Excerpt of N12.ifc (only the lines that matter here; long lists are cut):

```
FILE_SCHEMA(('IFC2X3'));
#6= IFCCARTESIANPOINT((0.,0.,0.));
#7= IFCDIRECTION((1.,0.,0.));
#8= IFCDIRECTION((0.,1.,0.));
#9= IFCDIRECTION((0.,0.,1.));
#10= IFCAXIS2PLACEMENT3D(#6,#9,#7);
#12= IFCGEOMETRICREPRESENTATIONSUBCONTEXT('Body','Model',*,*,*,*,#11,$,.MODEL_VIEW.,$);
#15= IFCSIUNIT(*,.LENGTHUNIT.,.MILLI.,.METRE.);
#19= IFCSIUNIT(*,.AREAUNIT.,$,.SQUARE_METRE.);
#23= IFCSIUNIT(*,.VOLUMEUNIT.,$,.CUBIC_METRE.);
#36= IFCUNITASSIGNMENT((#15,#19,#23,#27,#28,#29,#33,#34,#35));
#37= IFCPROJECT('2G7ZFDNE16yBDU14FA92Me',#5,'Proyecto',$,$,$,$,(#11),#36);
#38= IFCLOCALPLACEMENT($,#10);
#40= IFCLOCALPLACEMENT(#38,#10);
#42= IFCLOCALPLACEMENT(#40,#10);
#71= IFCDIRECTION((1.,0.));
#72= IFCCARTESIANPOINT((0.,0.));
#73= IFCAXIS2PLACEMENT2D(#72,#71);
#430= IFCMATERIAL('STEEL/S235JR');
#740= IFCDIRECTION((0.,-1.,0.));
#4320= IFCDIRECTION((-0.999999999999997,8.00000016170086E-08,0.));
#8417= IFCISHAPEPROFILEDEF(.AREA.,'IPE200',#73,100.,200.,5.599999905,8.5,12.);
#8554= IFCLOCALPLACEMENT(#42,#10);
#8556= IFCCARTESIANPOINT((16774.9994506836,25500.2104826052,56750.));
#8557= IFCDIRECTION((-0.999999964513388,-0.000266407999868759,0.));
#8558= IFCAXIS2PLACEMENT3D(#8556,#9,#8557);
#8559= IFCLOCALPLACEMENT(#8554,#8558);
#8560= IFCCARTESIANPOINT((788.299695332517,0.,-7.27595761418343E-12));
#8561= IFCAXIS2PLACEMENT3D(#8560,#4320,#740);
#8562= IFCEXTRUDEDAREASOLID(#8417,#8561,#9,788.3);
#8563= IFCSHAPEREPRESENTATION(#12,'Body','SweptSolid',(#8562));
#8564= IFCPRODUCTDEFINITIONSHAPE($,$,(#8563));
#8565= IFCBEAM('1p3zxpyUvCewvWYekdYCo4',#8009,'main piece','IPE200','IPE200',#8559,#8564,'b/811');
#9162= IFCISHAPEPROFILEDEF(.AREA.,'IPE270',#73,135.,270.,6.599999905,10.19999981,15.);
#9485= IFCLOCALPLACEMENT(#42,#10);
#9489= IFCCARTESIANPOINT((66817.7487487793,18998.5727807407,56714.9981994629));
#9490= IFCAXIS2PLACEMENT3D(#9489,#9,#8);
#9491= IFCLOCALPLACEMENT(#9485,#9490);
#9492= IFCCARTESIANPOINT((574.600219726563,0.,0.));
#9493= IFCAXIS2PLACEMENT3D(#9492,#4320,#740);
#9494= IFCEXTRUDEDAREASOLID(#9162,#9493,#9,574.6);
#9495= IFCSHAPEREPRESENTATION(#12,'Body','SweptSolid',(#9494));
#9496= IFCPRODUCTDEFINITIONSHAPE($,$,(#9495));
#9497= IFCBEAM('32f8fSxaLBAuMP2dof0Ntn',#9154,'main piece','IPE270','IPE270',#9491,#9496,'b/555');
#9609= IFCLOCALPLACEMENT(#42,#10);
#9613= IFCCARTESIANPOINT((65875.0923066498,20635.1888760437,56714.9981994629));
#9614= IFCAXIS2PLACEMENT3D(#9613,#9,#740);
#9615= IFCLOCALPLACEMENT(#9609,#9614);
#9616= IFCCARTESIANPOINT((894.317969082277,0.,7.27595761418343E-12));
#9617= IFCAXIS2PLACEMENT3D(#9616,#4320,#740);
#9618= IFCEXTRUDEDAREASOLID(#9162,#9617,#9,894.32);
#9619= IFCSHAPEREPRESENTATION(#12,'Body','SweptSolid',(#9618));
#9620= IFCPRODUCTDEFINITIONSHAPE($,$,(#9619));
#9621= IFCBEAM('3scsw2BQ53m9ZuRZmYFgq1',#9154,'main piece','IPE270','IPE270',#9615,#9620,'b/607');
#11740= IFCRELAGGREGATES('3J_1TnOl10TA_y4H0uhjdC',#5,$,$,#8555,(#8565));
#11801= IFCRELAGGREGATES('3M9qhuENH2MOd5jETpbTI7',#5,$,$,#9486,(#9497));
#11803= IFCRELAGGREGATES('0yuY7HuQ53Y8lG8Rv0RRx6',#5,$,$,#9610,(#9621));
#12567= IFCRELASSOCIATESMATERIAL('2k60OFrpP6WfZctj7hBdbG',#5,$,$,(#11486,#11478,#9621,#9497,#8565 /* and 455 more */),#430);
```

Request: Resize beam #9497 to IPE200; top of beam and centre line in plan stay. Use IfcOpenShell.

```python
import ifcopenshell
import ifcopenshell.util.element
import ifcopenshell.util.representation

model = ifcopenshell.open("N12.ifc")

member = model.by_guid("32f8fSxaLBAuMP2dof0Ntn")
source = next(p for p in model.by_type("IfcIShapeProfileDef") if p.ProfileName == "IPE200")

body = ifcopenshell.util.representation.get_representation(member, "Model", "Body")
solid = body.Items[0]
old_profile = solid.SweptArea

# Copy the section's sizes but keep this member's own profile position.
profile = ifcopenshell.util.element.copy(model, source)
# Profiles are centred, so shift by half the change in depth to hold the top.
shift = (old_profile.OverallDepth - profile.OverallDepth) / 2
x, y = old_profile.Position.Location.Coordinates
up = (0.0, 1.0)  # upwards, in the solid's own plane
location = model.createIfcCartesianPoint((x + up[0] * shift, y + up[1] * shift))
profile.Position = model.createIfcAxis2Placement2D(location, old_profile.Position.RefDirection)
solid.SweptArea = profile
if not model.get_total_inverses(old_profile):
    ifcopenshell.util.element.remove_deep2(model, old_profile)
member.Description = member.Description.replace("IPE270", "IPE200")
member.ObjectType = member.ObjectType.replace("IPE270", "IPE200")

print(solid.SweptArea)

model.write("N12_rev.ifc")
```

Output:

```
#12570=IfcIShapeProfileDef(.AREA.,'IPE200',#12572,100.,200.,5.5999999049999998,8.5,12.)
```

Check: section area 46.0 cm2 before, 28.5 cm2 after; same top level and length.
